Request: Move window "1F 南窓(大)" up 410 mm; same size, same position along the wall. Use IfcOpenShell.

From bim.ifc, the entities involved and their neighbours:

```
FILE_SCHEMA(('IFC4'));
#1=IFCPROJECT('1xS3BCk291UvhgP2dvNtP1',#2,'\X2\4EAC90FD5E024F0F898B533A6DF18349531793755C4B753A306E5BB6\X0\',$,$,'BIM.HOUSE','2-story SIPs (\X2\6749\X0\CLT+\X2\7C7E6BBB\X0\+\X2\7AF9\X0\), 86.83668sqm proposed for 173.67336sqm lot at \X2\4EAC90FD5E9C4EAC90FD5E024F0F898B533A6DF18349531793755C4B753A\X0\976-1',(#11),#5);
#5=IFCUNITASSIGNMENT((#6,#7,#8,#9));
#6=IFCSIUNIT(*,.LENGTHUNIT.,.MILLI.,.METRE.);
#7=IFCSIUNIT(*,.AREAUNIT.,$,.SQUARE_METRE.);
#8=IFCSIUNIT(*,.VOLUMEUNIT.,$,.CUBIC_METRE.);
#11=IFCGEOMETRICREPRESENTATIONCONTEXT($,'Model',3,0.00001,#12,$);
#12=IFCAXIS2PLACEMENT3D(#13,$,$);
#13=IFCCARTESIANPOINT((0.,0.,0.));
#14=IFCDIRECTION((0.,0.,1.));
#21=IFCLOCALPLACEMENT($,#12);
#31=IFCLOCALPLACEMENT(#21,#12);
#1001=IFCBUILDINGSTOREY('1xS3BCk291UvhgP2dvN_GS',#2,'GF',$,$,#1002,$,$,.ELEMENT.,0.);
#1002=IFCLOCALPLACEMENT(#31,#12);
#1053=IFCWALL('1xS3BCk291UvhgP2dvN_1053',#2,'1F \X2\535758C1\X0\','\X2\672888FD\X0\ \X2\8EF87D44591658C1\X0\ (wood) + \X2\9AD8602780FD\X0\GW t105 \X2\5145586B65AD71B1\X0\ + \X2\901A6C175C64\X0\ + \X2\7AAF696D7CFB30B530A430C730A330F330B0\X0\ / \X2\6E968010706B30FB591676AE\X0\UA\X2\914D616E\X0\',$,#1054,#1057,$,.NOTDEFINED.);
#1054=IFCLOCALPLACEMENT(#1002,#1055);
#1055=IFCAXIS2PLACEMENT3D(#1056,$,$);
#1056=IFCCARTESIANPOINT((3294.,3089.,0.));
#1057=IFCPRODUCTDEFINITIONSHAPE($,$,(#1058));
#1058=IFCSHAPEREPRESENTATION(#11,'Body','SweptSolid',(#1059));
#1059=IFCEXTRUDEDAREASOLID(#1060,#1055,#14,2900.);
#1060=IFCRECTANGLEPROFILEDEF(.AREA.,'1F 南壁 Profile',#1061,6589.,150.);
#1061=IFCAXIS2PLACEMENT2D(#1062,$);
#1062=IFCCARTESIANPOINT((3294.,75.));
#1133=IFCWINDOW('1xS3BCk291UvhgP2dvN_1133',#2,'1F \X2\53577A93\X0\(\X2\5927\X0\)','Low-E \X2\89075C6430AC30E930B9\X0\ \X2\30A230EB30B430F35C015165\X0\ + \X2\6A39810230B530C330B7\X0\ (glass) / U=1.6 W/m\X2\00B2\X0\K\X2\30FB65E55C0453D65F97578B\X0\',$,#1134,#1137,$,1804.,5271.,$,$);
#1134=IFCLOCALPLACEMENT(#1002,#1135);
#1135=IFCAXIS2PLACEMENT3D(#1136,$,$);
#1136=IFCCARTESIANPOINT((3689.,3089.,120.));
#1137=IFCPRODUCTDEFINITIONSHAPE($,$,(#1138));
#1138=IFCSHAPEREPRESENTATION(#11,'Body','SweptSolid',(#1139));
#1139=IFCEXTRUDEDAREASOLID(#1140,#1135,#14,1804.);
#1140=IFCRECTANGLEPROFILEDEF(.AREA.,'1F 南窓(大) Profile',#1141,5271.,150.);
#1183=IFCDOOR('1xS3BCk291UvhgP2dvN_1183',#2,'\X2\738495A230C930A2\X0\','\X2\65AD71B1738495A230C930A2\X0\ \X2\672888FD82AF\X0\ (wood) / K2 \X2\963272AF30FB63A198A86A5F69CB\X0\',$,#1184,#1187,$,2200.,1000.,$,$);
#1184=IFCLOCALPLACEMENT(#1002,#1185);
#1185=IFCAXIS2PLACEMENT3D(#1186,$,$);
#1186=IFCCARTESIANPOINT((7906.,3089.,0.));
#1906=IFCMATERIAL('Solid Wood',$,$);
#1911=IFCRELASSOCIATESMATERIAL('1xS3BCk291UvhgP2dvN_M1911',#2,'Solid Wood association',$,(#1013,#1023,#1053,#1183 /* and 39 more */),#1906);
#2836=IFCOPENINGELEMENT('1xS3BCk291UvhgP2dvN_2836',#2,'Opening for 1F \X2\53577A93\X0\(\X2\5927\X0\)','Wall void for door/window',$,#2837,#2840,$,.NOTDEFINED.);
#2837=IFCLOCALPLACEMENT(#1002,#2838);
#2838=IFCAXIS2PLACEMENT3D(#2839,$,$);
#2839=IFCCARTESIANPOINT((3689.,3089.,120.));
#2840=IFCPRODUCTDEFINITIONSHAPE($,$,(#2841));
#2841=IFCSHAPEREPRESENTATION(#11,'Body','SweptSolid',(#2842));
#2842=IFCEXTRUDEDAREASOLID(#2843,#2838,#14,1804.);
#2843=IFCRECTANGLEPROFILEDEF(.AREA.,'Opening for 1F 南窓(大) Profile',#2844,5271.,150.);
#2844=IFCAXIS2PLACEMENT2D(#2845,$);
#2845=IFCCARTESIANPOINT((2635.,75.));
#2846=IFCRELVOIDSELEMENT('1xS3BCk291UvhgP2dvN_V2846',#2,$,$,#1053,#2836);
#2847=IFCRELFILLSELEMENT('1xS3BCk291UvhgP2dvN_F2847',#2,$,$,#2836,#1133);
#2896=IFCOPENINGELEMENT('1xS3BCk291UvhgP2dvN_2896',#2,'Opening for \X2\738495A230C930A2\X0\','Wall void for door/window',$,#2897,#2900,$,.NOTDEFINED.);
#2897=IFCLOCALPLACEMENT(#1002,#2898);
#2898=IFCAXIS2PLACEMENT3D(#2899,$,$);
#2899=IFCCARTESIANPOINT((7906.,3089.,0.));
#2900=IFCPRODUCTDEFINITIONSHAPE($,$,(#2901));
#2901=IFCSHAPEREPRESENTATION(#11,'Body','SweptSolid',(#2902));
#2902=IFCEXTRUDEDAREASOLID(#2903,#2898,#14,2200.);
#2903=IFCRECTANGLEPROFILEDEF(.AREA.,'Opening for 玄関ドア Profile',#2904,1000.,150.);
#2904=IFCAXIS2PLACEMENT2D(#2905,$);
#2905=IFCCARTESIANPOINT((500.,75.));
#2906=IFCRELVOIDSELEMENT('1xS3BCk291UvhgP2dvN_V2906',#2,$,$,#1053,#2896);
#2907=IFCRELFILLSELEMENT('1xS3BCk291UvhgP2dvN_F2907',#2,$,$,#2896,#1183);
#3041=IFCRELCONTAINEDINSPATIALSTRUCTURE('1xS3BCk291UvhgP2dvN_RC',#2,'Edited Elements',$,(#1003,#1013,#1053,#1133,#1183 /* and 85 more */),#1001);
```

```python
import numpy as np
import ifcopenshell
import ifcopenshell.api.geometry
import ifcopenshell.util.placement
import ifcopenshell.util.unit

model = ifcopenshell.open("bim.ifc")
unit_scale = ifcopenshell.util.unit.calculate_unit_scale(model)

window = model.by_guid("1xS3BCk291UvhgP2dvN_1133")
opening = window.FillsVoids[0].RelatingOpeningElement
dz = 0.41 / unit_scale

shift = np.array([0.0, 0.0, dz])
# The window is not placed relative to its opening, so move both.
for product in (opening, window):
    matrix = ifcopenshell.util.placement.get_local_placement(product.ObjectPlacement)
    matrix[:3, 3] += shift
    ifcopenshell.api.geometry.edit_object_placement(model, product=product, matrix=matrix, is_si=False)

print(f"moved by {dz * unit_scale:+.3f} m")

model.write("bim_edited.ifc")
```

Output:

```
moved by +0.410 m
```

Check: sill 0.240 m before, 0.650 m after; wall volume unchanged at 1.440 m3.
